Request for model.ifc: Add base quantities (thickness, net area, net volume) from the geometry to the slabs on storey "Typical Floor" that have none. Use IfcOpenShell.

First a look at what the model holds.

```python
import ifcopenshell
import ifcopenshell.util.element
import ifcopenshell.util.unit

model = ifcopenshell.open("model.ifc")
print(model.schema)
for unit_type in ("LENGTHUNIT", "AREAUNIT", "VOLUMEUNIT"):
    print(unit_type, ifcopenshell.util.unit.calculate_unit_scale(model, unit_type))
storey = next(s for s in model.by_type("IfcBuildingStorey") if s.Name == "Typical Floor")
slabs = [e for e in ifcopenshell.util.element.get_decomposition(storey) if e.is_a("IfcSlab")]
for e in sorted(slabs, key=lambda e: e.id()):
    print(e.id(), e.is_a(), e.Name, list(ifcopenshell.util.element.get_psets(e, qtos_only=True)), sep=" | ")
```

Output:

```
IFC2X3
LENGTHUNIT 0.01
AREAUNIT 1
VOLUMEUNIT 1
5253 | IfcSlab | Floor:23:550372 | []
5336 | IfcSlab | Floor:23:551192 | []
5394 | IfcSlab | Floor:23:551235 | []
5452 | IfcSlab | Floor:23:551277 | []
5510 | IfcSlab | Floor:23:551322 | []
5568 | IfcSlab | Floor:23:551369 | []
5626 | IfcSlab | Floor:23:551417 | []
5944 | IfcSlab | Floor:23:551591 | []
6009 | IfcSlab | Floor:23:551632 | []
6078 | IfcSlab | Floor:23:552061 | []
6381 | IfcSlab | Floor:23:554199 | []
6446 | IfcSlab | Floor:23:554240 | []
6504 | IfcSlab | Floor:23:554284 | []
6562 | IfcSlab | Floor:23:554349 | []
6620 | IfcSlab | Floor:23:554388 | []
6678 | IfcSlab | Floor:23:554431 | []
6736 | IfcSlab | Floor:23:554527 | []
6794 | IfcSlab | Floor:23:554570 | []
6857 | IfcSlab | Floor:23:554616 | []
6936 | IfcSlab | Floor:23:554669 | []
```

```python
import ifcopenshell
import ifcopenshell.api.pset
import ifcopenshell.geom
import ifcopenshell.util.element
import ifcopenshell.util.shape
import ifcopenshell.util.unit

model = ifcopenshell.open("model.ifc")
unit_scale = ifcopenshell.util.unit.calculate_unit_scale(model)
area_scale = ifcopenshell.util.unit.calculate_unit_scale(model, "AREAUNIT")
volume_scale = ifcopenshell.util.unit.calculate_unit_scale(model, "VOLUMEUNIT")
settings = ifcopenshell.geom.settings()

storey = next(s for s in model.by_type("IfcBuildingStorey") if s.Name == "Typical Floor")
slabs = [e for e in ifcopenshell.util.element.get_decomposition(storey) if e.is_a("IfcSlab")]

for e in sorted(slabs, key=lambda e: e.id()):
    if ifcopenshell.util.element.get_psets(e, qtos_only=True, should_inherit=False):
        continue
    # Geometry comes back in metres, in the element's own axes.
    shape = ifcopenshell.geom.create_shape(settings, e)
    values = {
        "Width": ifcopenshell.util.shape.get_z(shape.geometry) / unit_scale,
        "NetArea": ifcopenshell.util.shape.get_footprint_area(shape.geometry) / area_scale,
        "NetVolume": ifcopenshell.util.shape.get_volume(shape.geometry) / volume_scale,
    }
    qto = ifcopenshell.api.pset.add_qto(model, product=e, name="BaseQuantities")
    ifcopenshell.api.pset.edit_qto(model, qto=qto, properties=values)
    print(e.id(), {k: round(v, 3) for k, v in values.items()})

model.write("model_rev.ifc")
```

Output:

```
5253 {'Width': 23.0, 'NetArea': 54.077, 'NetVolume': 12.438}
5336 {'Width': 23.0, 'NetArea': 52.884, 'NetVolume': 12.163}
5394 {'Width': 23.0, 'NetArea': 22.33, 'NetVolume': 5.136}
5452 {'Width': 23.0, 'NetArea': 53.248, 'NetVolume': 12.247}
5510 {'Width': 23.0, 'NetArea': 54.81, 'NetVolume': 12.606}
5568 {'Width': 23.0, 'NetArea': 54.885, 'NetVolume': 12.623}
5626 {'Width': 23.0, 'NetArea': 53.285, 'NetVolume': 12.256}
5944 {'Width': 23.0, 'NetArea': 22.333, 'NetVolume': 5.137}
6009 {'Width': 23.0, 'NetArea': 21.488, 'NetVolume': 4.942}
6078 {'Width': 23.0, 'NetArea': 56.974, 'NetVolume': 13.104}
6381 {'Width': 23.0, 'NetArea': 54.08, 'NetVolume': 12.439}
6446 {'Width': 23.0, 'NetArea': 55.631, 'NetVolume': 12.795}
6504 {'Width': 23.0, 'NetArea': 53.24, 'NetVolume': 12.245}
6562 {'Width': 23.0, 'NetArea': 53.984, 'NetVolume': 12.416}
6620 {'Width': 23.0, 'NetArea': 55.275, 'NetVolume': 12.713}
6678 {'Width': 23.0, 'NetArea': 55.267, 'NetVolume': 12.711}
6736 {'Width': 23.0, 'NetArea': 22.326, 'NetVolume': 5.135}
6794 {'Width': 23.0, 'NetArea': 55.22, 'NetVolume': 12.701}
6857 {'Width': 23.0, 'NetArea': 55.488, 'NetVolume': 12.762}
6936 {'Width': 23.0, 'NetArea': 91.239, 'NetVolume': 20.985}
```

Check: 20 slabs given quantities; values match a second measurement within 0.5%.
